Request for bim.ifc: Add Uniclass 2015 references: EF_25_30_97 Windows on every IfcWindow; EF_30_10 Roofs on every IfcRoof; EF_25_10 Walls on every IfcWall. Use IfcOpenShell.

First a look at what the model holds.

```python
import ifcopenshell

model = ifcopenshell.open("bim.ifc")
print(model.schema)
print("classifications:", [c.Name for c in model.by_type("IfcClassification")])
for ifc_class in ("IfcDoor", "IfcRoof", "IfcStair", "IfcWall", "IfcWindow"):
    print(ifc_class, len(model.by_type(ifc_class)))
```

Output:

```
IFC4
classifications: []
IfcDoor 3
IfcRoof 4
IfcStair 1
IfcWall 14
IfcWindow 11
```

```python
import ifcopenshell
import ifcopenshell.api.classification

model = ifcopenshell.open("bim.ifc")

system = ifcopenshell.api.classification.add_classification(model, classification="Uniclass 2015")

codes = {
    "IfcWindow": ("EF_25_30_97", "Windows"),
    "IfcRoof": ("EF_30_10", "Roofs"),
    "IfcWall": ("EF_25_10", "Walls"),
}
for ifc_class, (code, name) in codes.items():
    products = model.by_type(ifc_class)
    ifcopenshell.api.classification.add_reference(
        model, products=products, classification=system, identification=code, name=name
    )
    print(code, len(products))

model.write("bim_updated.ifc")
```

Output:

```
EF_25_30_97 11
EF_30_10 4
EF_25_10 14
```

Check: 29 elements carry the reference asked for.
